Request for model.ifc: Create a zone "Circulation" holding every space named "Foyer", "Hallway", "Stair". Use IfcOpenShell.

First a look at what the model holds.

```python
import ifcopenshell

model = ifcopenshell.open("model.ifc")
print(model.schema)
seen = {}
for space in model.by_type("IfcSpace"):
    seen[space.LongName] = seen.get(space.LongName, 0) + 1
for name, count in sorted(seen.items(), key=str):
    print(count, "x", name)
print("zones:", [z.Name for z in model.by_type("IfcZone")][:20])
```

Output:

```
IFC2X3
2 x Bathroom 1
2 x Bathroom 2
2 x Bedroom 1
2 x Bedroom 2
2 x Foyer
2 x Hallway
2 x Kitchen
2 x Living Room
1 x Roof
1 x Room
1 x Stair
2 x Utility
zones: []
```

```python
import ifcopenshell
import ifcopenshell.api.group
import ifcopenshell.api.root

model = ifcopenshell.open("model.ifc")

names = {"Foyer", "Hallway", "Stair"}
spaces = [s for s in model.by_type("IfcSpace") if s.LongName in names]

zone = ifcopenshell.api.root.create_entity(model, ifc_class="IfcZone", name="Circulation")
ifcopenshell.api.group.assign_group(model, products=spaces, group=zone)
print(len(spaces), "spaces in", zone.Name)

model.write("model_rev.ifc")
```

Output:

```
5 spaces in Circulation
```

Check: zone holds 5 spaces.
